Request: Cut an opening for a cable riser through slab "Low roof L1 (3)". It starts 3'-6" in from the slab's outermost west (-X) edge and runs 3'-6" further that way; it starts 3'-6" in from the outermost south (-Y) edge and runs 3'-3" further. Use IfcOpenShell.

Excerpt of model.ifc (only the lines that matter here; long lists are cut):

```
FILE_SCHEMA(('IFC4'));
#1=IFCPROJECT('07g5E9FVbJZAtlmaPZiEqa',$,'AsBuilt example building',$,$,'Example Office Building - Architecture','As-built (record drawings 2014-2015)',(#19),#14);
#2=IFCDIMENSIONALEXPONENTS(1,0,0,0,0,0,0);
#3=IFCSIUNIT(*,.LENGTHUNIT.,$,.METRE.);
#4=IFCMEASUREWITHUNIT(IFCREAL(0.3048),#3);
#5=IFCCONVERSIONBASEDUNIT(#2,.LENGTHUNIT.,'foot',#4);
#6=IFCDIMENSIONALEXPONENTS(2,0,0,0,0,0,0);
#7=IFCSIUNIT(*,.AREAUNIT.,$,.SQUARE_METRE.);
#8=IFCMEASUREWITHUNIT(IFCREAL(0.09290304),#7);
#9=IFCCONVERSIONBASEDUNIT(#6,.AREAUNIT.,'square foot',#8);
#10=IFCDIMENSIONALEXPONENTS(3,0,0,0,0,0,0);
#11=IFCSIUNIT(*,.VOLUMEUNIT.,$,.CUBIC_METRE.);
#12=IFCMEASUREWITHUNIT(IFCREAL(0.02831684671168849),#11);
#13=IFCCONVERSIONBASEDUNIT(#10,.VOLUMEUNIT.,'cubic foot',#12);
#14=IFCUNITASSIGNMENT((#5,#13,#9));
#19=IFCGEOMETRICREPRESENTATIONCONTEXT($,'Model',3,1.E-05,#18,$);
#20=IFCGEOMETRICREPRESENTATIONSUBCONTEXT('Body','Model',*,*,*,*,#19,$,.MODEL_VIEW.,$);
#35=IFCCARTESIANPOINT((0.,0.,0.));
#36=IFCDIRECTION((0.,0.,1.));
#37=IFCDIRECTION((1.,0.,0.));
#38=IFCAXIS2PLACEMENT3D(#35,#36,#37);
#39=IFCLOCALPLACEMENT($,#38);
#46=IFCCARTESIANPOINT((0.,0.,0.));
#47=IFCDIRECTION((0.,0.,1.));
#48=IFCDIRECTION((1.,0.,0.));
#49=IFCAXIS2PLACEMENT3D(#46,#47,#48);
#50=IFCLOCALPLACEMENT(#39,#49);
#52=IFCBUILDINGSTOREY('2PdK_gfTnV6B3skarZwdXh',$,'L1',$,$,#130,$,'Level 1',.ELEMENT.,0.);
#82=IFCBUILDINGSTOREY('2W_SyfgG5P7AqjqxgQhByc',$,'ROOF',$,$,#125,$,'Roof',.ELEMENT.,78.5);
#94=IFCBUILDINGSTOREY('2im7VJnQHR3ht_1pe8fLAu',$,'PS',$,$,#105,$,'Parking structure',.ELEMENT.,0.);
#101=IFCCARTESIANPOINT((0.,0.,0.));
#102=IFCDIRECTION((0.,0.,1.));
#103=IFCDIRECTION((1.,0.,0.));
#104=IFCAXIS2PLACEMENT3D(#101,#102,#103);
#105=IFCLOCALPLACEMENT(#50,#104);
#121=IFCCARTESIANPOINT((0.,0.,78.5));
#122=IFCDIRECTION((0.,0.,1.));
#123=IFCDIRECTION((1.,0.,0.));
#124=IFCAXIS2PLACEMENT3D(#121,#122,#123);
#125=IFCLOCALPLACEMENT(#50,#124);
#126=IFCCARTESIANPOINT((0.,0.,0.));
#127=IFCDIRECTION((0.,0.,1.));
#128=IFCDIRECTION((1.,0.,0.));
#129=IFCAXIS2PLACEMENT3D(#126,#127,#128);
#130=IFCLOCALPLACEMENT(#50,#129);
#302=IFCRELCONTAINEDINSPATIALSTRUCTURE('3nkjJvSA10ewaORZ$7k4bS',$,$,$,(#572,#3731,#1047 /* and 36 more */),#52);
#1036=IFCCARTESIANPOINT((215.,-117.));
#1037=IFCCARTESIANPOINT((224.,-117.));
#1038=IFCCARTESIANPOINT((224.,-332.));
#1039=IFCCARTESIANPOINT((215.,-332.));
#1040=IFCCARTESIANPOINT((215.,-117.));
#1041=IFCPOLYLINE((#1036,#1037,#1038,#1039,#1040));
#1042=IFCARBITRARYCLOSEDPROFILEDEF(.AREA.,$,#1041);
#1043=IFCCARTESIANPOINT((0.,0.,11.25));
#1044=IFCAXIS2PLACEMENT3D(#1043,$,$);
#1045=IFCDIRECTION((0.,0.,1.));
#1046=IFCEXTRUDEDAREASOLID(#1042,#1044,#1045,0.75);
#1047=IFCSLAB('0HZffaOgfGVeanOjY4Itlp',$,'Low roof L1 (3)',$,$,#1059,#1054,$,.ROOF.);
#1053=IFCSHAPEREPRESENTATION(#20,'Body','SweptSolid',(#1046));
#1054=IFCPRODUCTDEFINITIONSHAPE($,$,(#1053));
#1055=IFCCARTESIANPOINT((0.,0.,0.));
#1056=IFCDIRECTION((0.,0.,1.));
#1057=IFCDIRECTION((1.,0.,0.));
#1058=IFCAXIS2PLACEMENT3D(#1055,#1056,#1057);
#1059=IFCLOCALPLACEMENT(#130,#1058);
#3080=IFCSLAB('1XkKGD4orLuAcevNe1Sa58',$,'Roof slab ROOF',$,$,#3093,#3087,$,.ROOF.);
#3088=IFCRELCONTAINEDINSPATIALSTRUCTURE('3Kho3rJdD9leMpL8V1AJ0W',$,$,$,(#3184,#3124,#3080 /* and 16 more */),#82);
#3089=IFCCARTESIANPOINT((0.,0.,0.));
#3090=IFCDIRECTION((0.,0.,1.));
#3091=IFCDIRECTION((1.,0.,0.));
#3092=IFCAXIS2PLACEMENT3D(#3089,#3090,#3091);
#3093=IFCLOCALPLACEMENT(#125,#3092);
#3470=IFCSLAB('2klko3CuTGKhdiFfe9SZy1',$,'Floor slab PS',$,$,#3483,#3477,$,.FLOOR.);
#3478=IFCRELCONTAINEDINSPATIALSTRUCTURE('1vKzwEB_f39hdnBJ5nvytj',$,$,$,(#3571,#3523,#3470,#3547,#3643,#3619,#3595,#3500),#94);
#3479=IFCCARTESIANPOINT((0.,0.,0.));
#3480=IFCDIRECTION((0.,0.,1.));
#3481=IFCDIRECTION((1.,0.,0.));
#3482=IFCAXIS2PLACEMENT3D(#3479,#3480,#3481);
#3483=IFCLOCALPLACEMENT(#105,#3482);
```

```python
import numpy as np
import ifcopenshell
import ifcopenshell.api.feature
import ifcopenshell.api.geometry
import ifcopenshell.api.root
import ifcopenshell.geom
import ifcopenshell.util.placement
import ifcopenshell.util.representation
import ifcopenshell.util.shape
import ifcopenshell.util.unit

model = ifcopenshell.open("model.ifc")
unit_scale = ifcopenshell.util.unit.calculate_unit_scale(model)
settings = ifcopenshell.geom.settings()


def volume(element):
    """Net volume in cubic metres, openings subtracted."""
    shape = ifcopenshell.geom.create_shape(settings, element)
    return ifcopenshell.util.shape.get_volume(shape.geometry)


slab = model.by_guid("0HZffaOgfGVeanOjY4Itlp")
before = volume(slab)

# Extent in the slab's own axes, in metres. The edges named are its -X and -Y sides.
slab_shape = ifcopenshell.geom.create_shape(settings, slab)
vertices = ifcopenshell.util.shape.get_vertices(slab_shape.geometry)
x_min, y_min, bottom = vertices.min(axis=0)
top = vertices[:, 2].max()

opening = ifcopenshell.api.root.create_entity(model, ifc_class="IfcOpeningElement", name="Cable riser opening", predefined_type="OPENING")
context = ifcopenshell.util.representation.get_context(model, "Model", "Body", "MODEL_VIEW")
width, depth = 1.0668, 0.9906
outline = [(0.0, 0.0), (width, 0.0), (width, depth), (0.0, depth), (0.0, 0.0)]
# Overshoot both faces by 50 mm so the cut is clean.
shape = ifcopenshell.api.geometry.add_slab_representation(
    model, context=context, depth=top - bottom + 0.1, polyline=outline
)
ifcopenshell.api.geometry.assign_representation(model, product=opening, representation=shape)

matrix = ifcopenshell.util.placement.get_local_placement(slab.ObjectPlacement)
matrix[:, 3] = matrix @ np.append(np.array([x_min + 1.0668, y_min + 1.0668, bottom - 0.05]) / unit_scale, 1.0)
ifcopenshell.api.geometry.edit_object_placement(model, product=opening, matrix=matrix, is_si=False)
ifcopenshell.api.feature.add_feature(model, feature=opening, element=slab)

after = volume(slab)

print(f"slab volume {before:.3f} -> {after:.3f} m3")

model.write("model_updated.ifc")
```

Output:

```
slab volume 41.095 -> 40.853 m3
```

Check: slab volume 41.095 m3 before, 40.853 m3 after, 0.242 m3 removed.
